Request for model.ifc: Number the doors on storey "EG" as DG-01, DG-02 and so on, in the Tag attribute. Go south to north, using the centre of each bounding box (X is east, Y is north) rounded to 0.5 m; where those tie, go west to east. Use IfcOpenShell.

First a look at what the model holds.

```python
import ifcopenshell
import ifcopenshell.util.element
import ifcopenshell.util.placement

model = ifcopenshell.open("model.ifc")
print(model.schema)
storey = next(s for s in model.by_type("IfcBuildingStorey") if s.Name == "EG")
doors = [e for e in ifcopenshell.util.element.get_decomposition(storey) if e.is_a("IfcDoor")]
for e in sorted(doors, key=lambda e: e.id()):
    origin = ifcopenshell.util.placement.get_local_placement(e.ObjectPlacement)[:3, 3]
    print(e.id(), e.Tag, e.Name, origin.round(2) + 0.0, sep=" | ")
```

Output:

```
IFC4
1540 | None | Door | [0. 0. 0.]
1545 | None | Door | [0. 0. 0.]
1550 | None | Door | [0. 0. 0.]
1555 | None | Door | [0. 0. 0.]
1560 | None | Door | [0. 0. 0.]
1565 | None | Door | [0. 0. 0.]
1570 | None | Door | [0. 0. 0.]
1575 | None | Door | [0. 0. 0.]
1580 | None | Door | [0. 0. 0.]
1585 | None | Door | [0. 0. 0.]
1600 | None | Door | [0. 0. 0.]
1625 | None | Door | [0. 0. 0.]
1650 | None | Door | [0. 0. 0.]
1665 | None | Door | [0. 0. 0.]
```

```python
import ifcopenshell
import ifcopenshell.geom
import ifcopenshell.util.element
import ifcopenshell.util.shape

model = ifcopenshell.open("model.ifc")
settings = ifcopenshell.geom.settings()
settings.set("use-world-coords", True)


def centre(element):
    shape = ifcopenshell.geom.create_shape(settings, element)
    return ifcopenshell.util.shape.get_bbox_centroid(shape.geometry)


storey = next(s for s in model.by_type("IfcBuildingStorey") if s.Name == "EG")
doors = [e for e in ifcopenshell.util.element.get_decomposition(storey) if e.is_a("IfcDoor")]

# Insertion points can sit at a corner or the storey origin, so sort by the geometry (in metres).
centres = {e: centre(e) for e in doors}
doors.sort(key=lambda e: (round(centres[e][1] / 0.5), centres[e][0]))

for i, e in enumerate(doors, start=1):
    number = f"DG-{i:02d}"
    e.Tag = number
    print(e.id(), number)

model.write("model_v2.ifc")
```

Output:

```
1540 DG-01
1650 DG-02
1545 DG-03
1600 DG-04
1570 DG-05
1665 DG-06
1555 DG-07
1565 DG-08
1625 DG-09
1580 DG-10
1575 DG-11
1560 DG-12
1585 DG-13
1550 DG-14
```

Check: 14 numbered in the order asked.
